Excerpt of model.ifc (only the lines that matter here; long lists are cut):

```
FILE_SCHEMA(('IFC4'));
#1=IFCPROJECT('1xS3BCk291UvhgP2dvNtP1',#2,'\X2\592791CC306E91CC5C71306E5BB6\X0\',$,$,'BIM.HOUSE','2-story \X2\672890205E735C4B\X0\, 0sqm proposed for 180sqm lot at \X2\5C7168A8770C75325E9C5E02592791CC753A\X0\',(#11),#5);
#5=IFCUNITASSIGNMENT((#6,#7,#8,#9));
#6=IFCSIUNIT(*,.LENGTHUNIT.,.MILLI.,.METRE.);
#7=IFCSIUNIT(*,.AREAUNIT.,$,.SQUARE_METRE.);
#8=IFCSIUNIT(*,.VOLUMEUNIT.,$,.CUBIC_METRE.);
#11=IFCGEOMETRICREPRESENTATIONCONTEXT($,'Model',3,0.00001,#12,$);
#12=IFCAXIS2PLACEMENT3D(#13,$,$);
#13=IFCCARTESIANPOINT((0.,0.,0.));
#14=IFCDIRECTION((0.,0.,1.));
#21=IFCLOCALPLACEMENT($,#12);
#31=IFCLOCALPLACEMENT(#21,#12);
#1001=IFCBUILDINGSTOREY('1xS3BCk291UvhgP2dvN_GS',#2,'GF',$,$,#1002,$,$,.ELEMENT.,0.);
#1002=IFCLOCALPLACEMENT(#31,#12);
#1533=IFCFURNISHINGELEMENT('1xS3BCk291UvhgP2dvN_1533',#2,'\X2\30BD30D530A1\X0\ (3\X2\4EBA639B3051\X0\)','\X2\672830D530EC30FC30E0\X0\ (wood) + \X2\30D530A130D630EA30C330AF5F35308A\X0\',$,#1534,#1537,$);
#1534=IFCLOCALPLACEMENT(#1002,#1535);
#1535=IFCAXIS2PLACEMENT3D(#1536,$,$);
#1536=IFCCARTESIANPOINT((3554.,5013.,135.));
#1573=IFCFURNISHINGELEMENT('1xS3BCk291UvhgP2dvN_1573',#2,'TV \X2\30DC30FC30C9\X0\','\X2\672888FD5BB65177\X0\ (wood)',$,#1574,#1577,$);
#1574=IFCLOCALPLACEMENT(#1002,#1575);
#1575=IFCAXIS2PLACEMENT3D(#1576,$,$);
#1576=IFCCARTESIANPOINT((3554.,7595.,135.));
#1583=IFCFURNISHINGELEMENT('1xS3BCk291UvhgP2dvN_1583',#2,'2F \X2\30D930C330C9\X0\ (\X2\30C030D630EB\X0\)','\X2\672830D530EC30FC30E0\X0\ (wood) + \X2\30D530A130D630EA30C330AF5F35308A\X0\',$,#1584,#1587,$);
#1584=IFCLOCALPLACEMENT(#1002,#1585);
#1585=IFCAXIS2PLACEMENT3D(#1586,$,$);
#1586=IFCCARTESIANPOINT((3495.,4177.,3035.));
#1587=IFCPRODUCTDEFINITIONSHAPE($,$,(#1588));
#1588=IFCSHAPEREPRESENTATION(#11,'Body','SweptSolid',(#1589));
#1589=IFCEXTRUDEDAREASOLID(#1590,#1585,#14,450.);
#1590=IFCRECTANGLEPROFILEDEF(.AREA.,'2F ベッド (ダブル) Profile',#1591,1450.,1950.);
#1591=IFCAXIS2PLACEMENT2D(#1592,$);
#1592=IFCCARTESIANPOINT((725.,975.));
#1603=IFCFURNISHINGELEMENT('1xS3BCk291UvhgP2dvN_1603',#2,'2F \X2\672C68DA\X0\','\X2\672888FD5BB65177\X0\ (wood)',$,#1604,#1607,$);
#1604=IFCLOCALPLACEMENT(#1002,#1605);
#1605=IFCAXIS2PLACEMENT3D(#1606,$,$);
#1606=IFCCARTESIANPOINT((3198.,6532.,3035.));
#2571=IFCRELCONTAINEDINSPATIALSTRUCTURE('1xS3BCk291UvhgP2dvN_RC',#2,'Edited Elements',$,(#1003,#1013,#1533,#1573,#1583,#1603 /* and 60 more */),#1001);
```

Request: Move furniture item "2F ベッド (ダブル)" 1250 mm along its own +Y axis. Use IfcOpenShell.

```python
import ifcopenshell
import ifcopenshell.api.geometry
import ifcopenshell.util.placement
import ifcopenshell.util.unit

model = ifcopenshell.open("model.ifc")
unit_scale = ifcopenshell.util.unit.calculate_unit_scale(model)

item = model.by_guid("1xS3BCk291UvhgP2dvN_1583")
matrix = ifcopenshell.util.placement.get_local_placement(item.ObjectPlacement)
matrix[:3, 3] += matrix[:3, 1] * 1.25 / unit_scale
ifcopenshell.api.geometry.edit_object_placement(model, product=item, matrix=matrix, is_si=False)

print(ifcopenshell.util.placement.get_local_placement(item.ObjectPlacement).round(3) + 0.0)

model.write("model_updated.ifc")
```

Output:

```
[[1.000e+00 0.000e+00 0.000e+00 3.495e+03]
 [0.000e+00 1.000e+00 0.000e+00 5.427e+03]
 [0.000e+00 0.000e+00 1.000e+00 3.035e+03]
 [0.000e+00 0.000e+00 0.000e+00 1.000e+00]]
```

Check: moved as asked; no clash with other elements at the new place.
